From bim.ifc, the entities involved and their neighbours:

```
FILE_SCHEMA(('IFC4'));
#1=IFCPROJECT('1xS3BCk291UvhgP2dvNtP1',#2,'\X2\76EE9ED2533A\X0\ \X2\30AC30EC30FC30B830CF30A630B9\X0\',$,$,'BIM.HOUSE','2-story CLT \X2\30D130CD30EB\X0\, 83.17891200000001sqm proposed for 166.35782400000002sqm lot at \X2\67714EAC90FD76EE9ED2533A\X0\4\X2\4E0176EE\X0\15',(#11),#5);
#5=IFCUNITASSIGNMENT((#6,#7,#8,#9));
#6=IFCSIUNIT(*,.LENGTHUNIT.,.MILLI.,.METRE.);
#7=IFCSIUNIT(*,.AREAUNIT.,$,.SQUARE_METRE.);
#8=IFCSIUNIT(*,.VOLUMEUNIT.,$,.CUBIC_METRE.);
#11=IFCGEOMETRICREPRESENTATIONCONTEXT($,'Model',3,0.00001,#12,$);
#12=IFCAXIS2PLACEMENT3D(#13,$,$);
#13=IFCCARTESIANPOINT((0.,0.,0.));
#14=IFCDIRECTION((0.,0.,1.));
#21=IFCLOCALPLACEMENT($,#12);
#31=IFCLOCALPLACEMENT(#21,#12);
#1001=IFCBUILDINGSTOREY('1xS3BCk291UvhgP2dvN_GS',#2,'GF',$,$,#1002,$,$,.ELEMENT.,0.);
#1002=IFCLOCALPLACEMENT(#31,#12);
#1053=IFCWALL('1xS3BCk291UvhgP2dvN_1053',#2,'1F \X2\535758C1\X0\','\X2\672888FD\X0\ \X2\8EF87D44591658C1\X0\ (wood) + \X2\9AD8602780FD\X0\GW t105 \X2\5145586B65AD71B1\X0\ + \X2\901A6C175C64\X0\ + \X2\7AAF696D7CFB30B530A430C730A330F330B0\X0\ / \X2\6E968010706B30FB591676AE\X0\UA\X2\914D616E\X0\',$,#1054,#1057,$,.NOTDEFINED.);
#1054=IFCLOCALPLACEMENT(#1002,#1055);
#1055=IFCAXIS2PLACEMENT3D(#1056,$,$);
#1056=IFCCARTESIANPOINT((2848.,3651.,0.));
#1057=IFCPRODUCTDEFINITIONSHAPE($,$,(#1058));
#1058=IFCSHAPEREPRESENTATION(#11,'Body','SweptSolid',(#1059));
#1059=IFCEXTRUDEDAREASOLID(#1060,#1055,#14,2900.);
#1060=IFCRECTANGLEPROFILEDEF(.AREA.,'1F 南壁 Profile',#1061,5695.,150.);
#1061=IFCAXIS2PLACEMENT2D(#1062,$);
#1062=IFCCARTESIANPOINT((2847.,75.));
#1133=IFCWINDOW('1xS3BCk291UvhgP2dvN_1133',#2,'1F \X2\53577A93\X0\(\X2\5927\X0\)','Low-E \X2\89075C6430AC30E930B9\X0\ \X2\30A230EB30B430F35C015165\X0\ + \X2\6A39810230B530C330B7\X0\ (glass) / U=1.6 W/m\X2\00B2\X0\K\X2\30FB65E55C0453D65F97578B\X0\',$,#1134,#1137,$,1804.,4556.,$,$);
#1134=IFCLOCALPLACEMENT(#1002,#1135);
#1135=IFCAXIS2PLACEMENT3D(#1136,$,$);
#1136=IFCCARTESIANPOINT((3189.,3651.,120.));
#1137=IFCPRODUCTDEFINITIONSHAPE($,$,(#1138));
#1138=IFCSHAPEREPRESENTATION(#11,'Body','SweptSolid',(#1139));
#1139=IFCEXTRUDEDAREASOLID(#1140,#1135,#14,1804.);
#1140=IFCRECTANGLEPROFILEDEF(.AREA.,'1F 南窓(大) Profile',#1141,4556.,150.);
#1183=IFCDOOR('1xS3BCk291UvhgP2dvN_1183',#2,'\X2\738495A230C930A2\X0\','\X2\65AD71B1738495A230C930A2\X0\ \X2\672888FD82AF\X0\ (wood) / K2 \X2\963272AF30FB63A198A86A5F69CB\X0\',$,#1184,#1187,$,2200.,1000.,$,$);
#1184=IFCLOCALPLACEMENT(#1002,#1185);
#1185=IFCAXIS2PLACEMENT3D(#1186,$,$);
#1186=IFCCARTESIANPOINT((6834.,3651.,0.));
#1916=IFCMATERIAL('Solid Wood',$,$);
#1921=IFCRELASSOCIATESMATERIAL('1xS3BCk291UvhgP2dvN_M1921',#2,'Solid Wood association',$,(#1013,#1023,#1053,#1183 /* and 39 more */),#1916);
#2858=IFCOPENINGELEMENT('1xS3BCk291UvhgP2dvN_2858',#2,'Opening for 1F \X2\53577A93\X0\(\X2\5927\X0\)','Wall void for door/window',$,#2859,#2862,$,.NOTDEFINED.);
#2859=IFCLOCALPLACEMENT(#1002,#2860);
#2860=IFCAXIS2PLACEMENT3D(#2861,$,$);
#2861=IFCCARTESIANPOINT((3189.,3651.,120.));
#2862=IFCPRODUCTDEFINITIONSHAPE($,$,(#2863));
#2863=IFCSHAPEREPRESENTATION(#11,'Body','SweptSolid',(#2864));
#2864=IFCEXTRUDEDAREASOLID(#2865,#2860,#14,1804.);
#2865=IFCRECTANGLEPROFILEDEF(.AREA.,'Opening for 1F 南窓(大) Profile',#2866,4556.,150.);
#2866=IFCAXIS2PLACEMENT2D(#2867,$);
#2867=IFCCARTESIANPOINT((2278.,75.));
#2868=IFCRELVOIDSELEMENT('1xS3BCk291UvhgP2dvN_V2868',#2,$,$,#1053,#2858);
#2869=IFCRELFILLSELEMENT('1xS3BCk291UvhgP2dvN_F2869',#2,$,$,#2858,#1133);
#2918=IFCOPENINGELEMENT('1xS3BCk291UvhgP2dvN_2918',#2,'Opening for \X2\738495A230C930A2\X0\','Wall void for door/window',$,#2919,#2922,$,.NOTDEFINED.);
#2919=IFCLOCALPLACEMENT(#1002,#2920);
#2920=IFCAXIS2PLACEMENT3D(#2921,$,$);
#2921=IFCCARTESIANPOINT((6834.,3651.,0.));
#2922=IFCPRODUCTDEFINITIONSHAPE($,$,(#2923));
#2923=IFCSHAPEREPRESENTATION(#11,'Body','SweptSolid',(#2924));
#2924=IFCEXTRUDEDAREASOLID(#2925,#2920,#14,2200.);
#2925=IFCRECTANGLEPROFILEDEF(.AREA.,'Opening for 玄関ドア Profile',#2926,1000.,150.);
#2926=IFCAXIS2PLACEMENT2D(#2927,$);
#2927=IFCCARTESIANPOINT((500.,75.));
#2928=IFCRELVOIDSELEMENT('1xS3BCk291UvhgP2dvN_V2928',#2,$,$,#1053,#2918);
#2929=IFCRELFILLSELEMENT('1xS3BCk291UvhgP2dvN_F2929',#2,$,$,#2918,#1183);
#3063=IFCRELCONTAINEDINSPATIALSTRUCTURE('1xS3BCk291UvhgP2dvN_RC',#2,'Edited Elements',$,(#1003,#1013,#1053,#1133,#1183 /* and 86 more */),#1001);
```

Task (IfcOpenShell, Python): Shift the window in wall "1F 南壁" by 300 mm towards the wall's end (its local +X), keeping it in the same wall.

```python
import ifcopenshell
import ifcopenshell.api.geometry
import ifcopenshell.util.placement
import ifcopenshell.util.unit

model = ifcopenshell.open("bim.ifc")
unit_scale = ifcopenshell.util.unit.calculate_unit_scale(model)

window = model.by_id(1133)
opening = window.FillsVoids[0].RelatingOpeningElement
wall = opening.VoidsElements[0].RelatingBuildingElement

wall_matrix = ifcopenshell.util.placement.get_local_placement(wall.ObjectPlacement)
shift = wall_matrix[:3, 0] * 0.3 / unit_scale
before = ifcopenshell.util.placement.get_local_placement(window.ObjectPlacement)[:3, 3].copy()

# The window is not placed relative to its opening, so move both.
for product in (opening, window):
    matrix = ifcopenshell.util.placement.get_local_placement(product.ObjectPlacement)
    matrix[:3, 3] += shift
    ifcopenshell.api.geometry.edit_object_placement(model, product=product, matrix=matrix, is_si=False)

after = ifcopenshell.util.placement.get_local_placement(window.ObjectPlacement)[:3, 3]
print("window moved by", (after - before).round(3) + 0.0)

model.write("bim_rev.ifc")
```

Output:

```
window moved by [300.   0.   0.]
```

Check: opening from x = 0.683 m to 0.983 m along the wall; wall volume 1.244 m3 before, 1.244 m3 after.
